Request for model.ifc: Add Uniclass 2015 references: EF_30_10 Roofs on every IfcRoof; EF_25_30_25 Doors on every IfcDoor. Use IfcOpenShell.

First a look at what the model holds.

```python
import ifcopenshell

model = ifcopenshell.open("model.ifc")
print(model.schema)
print("classifications:", [c.Name for c in model.by_type("IfcClassification")])
for ifc_class in ("IfcDoor", "IfcRoof", "IfcStair", "IfcWall", "IfcWindow"):
    print(ifc_class, len(model.by_type(ifc_class)))
```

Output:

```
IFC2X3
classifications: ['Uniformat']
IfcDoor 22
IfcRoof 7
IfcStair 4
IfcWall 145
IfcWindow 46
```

```python
import ifcopenshell
import ifcopenshell.api.classification

model = ifcopenshell.open("model.ifc")

# IFC2X3 requires Source and Edition and has no link from the project to the system.
system = model.create_entity("IfcClassification", Source="NBS", Edition="2015", Name="Uniclass 2015")

codes = {
    "IfcRoof": ("EF_30_10", "Roofs"),
    "IfcDoor": ("EF_25_30_25", "Doors"),
}
for ifc_class, (code, name) in codes.items():
    products = model.by_type(ifc_class)
    ifcopenshell.api.classification.add_reference(
        model, products=products, classification=system, identification=code, name=name
    )
    print(code, len(products))

model.write("model_edited.ifc")
```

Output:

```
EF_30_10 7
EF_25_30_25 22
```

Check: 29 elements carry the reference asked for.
